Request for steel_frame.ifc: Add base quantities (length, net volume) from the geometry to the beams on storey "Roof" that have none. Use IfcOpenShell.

First a look at what the model holds.

```python
import ifcopenshell
import ifcopenshell.util.element
import ifcopenshell.util.unit

model = ifcopenshell.open("steel_frame.ifc")
print(model.schema)
for unit_type in ("LENGTHUNIT", "AREAUNIT", "VOLUMEUNIT"):
    print(unit_type, ifcopenshell.util.unit.calculate_unit_scale(model, unit_type))
storey = next(s for s in model.by_type("IfcBuildingStorey") if s.Name == "Roof")
beams = [e for e in ifcopenshell.util.element.get_decomposition(storey) if e.is_a("IfcBeam")]
for e in sorted(beams, key=lambda e: e.id()):
    print(e.id(), e.is_a(), e.Name, list(ifcopenshell.util.element.get_psets(e, qtos_only=True)), sep=" | ")
```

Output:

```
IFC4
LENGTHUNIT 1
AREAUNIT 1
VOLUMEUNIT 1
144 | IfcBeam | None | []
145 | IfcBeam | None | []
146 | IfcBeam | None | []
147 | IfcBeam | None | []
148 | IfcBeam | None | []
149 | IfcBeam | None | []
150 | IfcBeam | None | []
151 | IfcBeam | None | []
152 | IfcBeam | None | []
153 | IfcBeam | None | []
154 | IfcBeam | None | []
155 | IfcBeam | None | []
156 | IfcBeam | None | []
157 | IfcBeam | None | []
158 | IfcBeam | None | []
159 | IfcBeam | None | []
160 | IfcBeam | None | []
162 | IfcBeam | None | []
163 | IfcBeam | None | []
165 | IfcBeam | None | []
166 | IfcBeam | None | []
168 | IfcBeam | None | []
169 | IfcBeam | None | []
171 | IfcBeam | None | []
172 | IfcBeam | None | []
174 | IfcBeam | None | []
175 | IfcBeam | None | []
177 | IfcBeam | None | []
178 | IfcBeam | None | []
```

```python
import ifcopenshell
import ifcopenshell.api.pset
import ifcopenshell.geom
import ifcopenshell.util.element
import ifcopenshell.util.shape
import ifcopenshell.util.unit

model = ifcopenshell.open("steel_frame.ifc")
unit_scale = ifcopenshell.util.unit.calculate_unit_scale(model)
volume_scale = ifcopenshell.util.unit.calculate_unit_scale(model, "VOLUMEUNIT")
settings = ifcopenshell.geom.settings()

storey = next(s for s in model.by_type("IfcBuildingStorey") if s.Name == "Roof")
beams = [e for e in ifcopenshell.util.element.get_decomposition(storey) if e.is_a("IfcBeam")]

for e in sorted(beams, key=lambda e: e.id()):
    if ifcopenshell.util.element.get_psets(e, qtos_only=True, should_inherit=False):
        continue
    # Geometry comes back in metres, in the element's own axes.
    shape = ifcopenshell.geom.create_shape(settings, e)
    values = {
        "Length": ifcopenshell.util.shape.get_max_xyz(shape.geometry) / unit_scale,
        "NetVolume": ifcopenshell.util.shape.get_volume(shape.geometry) / volume_scale,
    }
    qto = ifcopenshell.api.pset.add_qto(model, product=e, name="Qto_BeamBaseQuantities")
    ifcopenshell.api.pset.edit_qto(model, qto=qto, properties=values)
    print(e.id(), {k: round(v, 3) for k, v in values.items()})

model.write("steel_frame_v2.ifc")
```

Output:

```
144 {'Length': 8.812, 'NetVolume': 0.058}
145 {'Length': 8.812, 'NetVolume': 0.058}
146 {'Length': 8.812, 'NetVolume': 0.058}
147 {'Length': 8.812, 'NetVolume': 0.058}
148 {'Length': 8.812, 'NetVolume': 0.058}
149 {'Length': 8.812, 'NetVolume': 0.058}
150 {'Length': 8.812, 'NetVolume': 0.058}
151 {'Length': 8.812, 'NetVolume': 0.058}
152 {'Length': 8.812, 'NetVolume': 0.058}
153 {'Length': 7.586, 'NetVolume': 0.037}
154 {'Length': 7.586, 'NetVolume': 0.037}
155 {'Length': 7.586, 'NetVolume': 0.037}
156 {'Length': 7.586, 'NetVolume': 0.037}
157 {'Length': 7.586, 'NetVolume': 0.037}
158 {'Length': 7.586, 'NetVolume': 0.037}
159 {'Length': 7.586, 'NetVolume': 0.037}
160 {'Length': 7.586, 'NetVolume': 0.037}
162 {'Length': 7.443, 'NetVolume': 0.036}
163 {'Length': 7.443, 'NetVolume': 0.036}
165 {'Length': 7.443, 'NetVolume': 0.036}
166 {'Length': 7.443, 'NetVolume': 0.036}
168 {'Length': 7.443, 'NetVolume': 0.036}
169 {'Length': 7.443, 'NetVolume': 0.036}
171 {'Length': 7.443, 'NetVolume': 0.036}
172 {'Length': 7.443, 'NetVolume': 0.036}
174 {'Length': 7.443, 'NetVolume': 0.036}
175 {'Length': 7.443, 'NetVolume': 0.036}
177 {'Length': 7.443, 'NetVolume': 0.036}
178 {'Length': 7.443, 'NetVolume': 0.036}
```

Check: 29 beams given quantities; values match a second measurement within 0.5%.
